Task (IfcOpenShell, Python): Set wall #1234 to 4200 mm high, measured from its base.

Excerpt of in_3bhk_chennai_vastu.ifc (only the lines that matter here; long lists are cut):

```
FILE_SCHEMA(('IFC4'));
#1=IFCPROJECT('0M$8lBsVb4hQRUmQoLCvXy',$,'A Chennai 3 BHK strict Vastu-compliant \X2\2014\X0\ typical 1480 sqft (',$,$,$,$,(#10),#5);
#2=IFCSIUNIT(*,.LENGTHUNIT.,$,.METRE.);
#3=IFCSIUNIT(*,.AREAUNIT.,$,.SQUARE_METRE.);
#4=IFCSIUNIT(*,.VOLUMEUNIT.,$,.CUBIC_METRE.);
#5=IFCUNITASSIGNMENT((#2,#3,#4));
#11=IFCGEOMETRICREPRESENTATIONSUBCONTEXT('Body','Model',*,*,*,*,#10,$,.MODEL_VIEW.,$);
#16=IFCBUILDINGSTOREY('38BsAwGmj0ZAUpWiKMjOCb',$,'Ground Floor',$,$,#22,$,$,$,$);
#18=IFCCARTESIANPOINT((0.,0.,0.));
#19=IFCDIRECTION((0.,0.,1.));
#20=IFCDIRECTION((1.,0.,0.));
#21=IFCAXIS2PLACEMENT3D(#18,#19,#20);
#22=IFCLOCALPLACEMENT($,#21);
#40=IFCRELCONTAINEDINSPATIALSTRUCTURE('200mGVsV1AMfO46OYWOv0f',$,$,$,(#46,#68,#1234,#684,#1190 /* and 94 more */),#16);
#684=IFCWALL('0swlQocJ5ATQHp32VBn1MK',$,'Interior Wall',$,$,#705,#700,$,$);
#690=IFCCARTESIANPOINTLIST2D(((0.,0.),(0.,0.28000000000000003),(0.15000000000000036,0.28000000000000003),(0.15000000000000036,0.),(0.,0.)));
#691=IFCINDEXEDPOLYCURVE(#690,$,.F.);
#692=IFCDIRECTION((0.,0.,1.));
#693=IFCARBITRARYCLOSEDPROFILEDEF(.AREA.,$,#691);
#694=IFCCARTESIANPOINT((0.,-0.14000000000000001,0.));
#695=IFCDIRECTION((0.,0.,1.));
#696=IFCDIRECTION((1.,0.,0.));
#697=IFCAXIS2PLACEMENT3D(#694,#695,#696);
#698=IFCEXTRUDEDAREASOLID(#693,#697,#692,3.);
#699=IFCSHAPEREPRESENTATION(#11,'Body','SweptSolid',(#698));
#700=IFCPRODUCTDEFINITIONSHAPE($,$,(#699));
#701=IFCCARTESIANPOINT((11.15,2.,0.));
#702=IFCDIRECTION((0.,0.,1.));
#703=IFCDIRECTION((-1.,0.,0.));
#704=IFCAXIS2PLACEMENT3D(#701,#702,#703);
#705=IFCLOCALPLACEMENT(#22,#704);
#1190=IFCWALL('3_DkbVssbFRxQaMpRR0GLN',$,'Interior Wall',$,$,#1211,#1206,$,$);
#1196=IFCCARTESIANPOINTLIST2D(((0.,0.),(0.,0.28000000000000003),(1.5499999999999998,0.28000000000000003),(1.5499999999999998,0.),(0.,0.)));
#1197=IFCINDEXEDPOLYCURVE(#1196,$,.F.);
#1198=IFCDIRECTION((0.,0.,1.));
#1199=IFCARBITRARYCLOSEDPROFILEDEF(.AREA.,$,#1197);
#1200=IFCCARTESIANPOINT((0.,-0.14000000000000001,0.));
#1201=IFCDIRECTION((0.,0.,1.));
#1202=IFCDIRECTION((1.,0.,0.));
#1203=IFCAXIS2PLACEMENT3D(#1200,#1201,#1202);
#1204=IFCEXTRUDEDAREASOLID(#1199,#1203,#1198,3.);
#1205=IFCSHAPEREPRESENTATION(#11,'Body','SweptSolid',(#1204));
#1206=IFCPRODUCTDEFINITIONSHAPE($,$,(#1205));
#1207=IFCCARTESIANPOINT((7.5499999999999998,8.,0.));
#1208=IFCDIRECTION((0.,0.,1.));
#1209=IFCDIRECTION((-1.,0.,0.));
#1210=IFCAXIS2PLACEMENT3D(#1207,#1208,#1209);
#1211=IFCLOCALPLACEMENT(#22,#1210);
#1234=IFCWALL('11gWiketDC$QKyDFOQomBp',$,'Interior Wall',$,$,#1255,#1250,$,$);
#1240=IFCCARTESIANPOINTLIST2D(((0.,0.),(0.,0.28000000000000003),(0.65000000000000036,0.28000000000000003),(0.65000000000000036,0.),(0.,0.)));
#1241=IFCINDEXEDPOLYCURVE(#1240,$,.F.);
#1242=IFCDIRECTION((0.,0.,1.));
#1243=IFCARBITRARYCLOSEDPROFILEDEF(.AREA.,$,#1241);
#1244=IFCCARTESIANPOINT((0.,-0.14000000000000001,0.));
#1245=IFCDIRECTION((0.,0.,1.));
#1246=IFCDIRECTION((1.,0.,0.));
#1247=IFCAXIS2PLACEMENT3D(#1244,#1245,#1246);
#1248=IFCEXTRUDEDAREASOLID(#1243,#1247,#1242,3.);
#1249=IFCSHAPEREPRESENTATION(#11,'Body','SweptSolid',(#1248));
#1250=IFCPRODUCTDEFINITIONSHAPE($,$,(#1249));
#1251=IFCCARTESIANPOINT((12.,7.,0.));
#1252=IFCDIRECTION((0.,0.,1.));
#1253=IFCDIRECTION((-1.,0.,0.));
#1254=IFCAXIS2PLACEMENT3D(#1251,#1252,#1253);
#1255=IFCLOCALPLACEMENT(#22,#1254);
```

```python
import ifcopenshell
import ifcopenshell.geom
import ifcopenshell.util.representation
import ifcopenshell.util.shape
import ifcopenshell.util.unit

model = ifcopenshell.open("in_3bhk_chennai_vastu.ifc")
unit_scale = ifcopenshell.util.unit.calculate_unit_scale(model)
settings = ifcopenshell.geom.settings()


def volume(element):
    """Net volume in cubic metres, openings subtracted."""
    shape = ifcopenshell.geom.create_shape(settings, element)
    return ifcopenshell.util.shape.get_volume(shape.geometry)


wall = model.by_id(1234)
before = volume(wall)

body = ifcopenshell.util.representation.get_representation(wall, "Model", "Body")
solid = body.Items[0]
old_height = solid.Depth
solid.Depth = 4.2 / unit_scale
after = volume(wall)

print(f"height {old_height:g} -> {solid.Depth:g}, volume {before:.3f} -> {after:.3f} m3")

model.write("in_3bhk_chennai_vastu_rev.ifc")
```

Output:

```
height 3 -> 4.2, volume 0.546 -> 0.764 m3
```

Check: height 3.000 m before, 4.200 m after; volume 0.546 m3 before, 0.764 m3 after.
